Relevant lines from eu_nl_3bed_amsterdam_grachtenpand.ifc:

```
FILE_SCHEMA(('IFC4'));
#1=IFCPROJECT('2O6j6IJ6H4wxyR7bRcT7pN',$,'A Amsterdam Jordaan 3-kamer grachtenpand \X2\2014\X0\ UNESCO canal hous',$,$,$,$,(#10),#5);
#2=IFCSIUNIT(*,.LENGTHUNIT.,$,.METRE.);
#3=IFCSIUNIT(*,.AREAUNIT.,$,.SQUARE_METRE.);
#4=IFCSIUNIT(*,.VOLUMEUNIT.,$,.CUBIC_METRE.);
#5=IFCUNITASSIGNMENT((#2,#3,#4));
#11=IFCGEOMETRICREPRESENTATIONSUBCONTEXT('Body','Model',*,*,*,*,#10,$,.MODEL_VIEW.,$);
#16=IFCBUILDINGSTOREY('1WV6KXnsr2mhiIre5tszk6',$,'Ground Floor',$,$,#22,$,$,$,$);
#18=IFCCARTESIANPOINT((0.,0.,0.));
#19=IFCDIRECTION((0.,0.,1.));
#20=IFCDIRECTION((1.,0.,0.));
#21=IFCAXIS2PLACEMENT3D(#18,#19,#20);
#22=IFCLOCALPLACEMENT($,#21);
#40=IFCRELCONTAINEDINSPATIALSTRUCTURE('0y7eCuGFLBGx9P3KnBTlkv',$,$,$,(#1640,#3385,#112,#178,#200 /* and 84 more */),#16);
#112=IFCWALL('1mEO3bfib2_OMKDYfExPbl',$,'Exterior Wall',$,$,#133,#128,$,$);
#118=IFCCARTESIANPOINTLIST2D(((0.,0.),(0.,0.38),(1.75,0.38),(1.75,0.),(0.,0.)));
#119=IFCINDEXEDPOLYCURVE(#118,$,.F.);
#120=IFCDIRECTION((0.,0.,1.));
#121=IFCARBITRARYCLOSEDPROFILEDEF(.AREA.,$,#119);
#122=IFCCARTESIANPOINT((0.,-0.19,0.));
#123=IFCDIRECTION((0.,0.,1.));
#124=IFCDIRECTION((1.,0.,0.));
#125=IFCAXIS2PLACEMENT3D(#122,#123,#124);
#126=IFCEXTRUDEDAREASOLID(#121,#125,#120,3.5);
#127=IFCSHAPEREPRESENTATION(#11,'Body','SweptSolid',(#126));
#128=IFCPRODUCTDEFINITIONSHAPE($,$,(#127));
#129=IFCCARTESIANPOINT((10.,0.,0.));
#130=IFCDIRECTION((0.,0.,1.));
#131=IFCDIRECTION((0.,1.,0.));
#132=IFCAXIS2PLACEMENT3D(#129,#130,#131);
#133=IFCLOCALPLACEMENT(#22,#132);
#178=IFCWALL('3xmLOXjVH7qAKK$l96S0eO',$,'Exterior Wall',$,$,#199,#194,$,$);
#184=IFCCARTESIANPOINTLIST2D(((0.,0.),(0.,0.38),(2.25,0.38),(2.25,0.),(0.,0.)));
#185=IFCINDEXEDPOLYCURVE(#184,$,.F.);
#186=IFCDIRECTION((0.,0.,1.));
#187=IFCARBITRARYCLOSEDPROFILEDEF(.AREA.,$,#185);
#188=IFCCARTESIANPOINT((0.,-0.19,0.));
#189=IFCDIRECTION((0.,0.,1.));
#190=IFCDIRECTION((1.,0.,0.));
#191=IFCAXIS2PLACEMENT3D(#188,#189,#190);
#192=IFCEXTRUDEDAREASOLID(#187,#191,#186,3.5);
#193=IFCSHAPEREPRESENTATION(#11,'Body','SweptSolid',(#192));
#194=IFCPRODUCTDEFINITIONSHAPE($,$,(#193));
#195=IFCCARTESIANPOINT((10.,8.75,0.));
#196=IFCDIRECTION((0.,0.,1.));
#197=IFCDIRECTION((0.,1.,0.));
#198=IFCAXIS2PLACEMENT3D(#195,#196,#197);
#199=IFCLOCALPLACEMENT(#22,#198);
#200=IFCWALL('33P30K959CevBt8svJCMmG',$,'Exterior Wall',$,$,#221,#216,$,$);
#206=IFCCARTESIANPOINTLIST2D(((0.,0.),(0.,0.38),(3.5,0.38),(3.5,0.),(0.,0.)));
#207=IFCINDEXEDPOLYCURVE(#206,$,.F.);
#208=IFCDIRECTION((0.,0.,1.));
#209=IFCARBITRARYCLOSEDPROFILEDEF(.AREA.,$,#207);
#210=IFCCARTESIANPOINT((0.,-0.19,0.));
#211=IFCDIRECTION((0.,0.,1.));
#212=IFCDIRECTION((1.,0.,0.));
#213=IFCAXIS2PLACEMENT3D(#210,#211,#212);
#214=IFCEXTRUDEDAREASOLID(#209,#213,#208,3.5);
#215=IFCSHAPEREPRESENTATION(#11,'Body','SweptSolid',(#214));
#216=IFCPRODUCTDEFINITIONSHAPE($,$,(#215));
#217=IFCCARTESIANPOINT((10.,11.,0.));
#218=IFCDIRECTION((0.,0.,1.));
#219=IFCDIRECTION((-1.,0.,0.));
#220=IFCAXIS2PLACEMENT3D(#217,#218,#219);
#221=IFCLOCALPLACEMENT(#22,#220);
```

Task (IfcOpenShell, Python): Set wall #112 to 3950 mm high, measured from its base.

```python
import ifcopenshell
import ifcopenshell.geom
import ifcopenshell.util.representation
import ifcopenshell.util.shape
import ifcopenshell.util.unit

model = ifcopenshell.open("eu_nl_3bed_amsterdam_grachtenpand.ifc")
unit_scale = ifcopenshell.util.unit.calculate_unit_scale(model)
settings = ifcopenshell.geom.settings()


def volume(element):
    """Net volume in cubic metres, openings subtracted."""
    shape = ifcopenshell.geom.create_shape(settings, element)
    return ifcopenshell.util.shape.get_volume(shape.geometry)


wall = model.by_id(112)
before = volume(wall)

body = ifcopenshell.util.representation.get_representation(wall, "Model", "Body")
solid = body.Items[0]
old_height = solid.Depth
solid.Depth = 3.95 / unit_scale
after = volume(wall)

print(f"height {old_height:g} -> {solid.Depth:g}, volume {before:.3f} -> {after:.3f} m3")

model.write("eu_nl_3bed_amsterdam_grachtenpand_v2.ifc")
```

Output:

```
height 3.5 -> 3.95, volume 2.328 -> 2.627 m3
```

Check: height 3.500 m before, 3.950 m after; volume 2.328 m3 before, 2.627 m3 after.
